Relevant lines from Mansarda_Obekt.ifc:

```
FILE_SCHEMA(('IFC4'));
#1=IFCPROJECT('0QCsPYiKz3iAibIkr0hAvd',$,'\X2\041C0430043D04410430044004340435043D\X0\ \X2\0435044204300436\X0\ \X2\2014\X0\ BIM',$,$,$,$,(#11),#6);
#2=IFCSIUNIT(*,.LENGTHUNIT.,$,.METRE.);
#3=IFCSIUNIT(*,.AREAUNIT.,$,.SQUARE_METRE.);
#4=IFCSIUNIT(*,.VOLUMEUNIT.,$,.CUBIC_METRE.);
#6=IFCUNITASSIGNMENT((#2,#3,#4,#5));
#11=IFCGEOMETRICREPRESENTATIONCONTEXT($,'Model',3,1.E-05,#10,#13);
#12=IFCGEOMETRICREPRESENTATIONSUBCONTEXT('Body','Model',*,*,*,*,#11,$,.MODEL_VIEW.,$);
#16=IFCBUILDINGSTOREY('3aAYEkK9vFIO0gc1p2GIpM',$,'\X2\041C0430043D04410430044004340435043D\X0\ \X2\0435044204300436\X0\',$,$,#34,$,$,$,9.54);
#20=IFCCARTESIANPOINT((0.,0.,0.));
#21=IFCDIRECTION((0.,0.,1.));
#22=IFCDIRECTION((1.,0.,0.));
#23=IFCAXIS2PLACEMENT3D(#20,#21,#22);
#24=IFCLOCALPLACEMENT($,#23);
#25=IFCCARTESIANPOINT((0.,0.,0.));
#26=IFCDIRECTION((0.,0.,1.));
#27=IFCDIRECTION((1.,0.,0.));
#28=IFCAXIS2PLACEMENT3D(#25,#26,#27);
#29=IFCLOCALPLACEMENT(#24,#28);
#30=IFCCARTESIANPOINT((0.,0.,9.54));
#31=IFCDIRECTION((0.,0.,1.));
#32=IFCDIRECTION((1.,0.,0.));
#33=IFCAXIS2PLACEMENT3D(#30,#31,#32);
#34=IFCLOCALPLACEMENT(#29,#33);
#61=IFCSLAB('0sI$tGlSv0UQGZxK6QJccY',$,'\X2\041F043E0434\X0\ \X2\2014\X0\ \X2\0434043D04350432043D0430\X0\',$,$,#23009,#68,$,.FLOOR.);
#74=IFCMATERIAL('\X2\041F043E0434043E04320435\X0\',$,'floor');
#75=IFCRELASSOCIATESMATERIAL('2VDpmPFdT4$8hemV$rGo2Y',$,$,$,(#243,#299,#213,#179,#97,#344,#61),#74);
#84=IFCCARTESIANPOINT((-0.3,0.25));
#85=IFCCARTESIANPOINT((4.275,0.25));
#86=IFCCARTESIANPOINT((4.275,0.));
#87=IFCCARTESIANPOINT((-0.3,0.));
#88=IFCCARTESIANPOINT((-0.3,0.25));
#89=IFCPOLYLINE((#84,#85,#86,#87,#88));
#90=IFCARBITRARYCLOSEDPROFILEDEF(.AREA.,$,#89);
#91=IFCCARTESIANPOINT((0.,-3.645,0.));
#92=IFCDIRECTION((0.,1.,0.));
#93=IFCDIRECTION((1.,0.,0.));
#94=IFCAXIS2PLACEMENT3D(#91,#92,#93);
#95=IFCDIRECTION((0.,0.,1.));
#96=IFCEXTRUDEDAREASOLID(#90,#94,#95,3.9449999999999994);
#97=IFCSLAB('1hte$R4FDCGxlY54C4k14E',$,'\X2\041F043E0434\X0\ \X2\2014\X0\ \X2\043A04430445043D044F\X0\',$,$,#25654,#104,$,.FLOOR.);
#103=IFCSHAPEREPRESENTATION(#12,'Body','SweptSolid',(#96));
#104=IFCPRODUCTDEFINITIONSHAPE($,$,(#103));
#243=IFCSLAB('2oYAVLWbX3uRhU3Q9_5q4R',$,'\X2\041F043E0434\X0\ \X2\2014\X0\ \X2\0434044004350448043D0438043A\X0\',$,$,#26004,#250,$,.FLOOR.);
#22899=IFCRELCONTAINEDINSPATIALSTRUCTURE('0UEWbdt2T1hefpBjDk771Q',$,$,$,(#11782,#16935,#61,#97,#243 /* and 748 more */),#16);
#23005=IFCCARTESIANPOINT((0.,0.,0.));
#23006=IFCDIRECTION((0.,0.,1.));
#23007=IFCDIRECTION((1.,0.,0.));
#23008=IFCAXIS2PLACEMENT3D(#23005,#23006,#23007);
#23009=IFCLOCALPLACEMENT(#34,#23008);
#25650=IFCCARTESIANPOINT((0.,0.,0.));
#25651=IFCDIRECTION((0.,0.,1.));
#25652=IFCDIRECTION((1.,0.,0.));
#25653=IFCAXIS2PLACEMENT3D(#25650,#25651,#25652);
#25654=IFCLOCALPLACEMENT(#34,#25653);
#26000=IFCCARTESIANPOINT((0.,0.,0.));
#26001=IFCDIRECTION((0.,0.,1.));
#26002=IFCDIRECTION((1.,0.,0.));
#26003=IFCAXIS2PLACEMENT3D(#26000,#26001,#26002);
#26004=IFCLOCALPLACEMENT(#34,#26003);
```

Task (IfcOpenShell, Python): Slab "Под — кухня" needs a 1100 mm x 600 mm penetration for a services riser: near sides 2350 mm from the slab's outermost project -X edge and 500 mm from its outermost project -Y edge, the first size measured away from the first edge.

```python
import numpy as np
import ifcopenshell
import ifcopenshell.api.feature
import ifcopenshell.api.geometry
import ifcopenshell.api.root
import ifcopenshell.geom
import ifcopenshell.util.placement
import ifcopenshell.util.representation
import ifcopenshell.util.shape
import ifcopenshell.util.unit

model = ifcopenshell.open("Mansarda_Obekt.ifc")
unit_scale = ifcopenshell.util.unit.calculate_unit_scale(model)
settings = ifcopenshell.geom.settings()


def volume(element):
    """Net volume in cubic metres, openings subtracted."""
    shape = ifcopenshell.geom.create_shape(settings, element)
    return ifcopenshell.util.shape.get_volume(shape.geometry)


slab = model.by_guid("1hte$R4FDCGxlY54C4k14E")
before = volume(slab)

# Extent in the slab's own axes, in metres. The edges named are its -X and -Y sides.
slab_shape = ifcopenshell.geom.create_shape(settings, slab)
vertices = ifcopenshell.util.shape.get_vertices(slab_shape.geometry)
x_min, y_min, bottom = vertices.min(axis=0)
top = vertices[:, 2].max()

opening = ifcopenshell.api.root.create_entity(model, ifc_class="IfcOpeningElement", name="Services riser opening", predefined_type="OPENING")
context = ifcopenshell.util.representation.get_context(model, "Model", "Body", "MODEL_VIEW")
width, depth = 1.1, 0.6
outline = [(0.0, 0.0), (width, 0.0), (width, depth), (0.0, depth), (0.0, 0.0)]
# Overshoot both faces by 50 mm so the cut is clean.
shape = ifcopenshell.api.geometry.add_slab_representation(
    model, context=context, depth=top - bottom + 0.1, polyline=outline
)
ifcopenshell.api.geometry.assign_representation(model, product=opening, representation=shape)

matrix = ifcopenshell.util.placement.get_local_placement(slab.ObjectPlacement)
matrix[:, 3] = matrix @ np.append(np.array([x_min + 2.35, y_min + 0.5, bottom - 0.05]) / unit_scale, 1.0)
ifcopenshell.api.geometry.edit_object_placement(model, product=opening, matrix=matrix, is_si=False)
ifcopenshell.api.feature.add_feature(model, feature=opening, element=slab)

after = volume(slab)

print(f"slab volume {before:.3f} -> {after:.3f} m3")

model.write("Mansarda_Obekt_rev.ifc")
```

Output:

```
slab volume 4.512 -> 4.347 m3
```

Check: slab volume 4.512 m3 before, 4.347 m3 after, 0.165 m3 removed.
